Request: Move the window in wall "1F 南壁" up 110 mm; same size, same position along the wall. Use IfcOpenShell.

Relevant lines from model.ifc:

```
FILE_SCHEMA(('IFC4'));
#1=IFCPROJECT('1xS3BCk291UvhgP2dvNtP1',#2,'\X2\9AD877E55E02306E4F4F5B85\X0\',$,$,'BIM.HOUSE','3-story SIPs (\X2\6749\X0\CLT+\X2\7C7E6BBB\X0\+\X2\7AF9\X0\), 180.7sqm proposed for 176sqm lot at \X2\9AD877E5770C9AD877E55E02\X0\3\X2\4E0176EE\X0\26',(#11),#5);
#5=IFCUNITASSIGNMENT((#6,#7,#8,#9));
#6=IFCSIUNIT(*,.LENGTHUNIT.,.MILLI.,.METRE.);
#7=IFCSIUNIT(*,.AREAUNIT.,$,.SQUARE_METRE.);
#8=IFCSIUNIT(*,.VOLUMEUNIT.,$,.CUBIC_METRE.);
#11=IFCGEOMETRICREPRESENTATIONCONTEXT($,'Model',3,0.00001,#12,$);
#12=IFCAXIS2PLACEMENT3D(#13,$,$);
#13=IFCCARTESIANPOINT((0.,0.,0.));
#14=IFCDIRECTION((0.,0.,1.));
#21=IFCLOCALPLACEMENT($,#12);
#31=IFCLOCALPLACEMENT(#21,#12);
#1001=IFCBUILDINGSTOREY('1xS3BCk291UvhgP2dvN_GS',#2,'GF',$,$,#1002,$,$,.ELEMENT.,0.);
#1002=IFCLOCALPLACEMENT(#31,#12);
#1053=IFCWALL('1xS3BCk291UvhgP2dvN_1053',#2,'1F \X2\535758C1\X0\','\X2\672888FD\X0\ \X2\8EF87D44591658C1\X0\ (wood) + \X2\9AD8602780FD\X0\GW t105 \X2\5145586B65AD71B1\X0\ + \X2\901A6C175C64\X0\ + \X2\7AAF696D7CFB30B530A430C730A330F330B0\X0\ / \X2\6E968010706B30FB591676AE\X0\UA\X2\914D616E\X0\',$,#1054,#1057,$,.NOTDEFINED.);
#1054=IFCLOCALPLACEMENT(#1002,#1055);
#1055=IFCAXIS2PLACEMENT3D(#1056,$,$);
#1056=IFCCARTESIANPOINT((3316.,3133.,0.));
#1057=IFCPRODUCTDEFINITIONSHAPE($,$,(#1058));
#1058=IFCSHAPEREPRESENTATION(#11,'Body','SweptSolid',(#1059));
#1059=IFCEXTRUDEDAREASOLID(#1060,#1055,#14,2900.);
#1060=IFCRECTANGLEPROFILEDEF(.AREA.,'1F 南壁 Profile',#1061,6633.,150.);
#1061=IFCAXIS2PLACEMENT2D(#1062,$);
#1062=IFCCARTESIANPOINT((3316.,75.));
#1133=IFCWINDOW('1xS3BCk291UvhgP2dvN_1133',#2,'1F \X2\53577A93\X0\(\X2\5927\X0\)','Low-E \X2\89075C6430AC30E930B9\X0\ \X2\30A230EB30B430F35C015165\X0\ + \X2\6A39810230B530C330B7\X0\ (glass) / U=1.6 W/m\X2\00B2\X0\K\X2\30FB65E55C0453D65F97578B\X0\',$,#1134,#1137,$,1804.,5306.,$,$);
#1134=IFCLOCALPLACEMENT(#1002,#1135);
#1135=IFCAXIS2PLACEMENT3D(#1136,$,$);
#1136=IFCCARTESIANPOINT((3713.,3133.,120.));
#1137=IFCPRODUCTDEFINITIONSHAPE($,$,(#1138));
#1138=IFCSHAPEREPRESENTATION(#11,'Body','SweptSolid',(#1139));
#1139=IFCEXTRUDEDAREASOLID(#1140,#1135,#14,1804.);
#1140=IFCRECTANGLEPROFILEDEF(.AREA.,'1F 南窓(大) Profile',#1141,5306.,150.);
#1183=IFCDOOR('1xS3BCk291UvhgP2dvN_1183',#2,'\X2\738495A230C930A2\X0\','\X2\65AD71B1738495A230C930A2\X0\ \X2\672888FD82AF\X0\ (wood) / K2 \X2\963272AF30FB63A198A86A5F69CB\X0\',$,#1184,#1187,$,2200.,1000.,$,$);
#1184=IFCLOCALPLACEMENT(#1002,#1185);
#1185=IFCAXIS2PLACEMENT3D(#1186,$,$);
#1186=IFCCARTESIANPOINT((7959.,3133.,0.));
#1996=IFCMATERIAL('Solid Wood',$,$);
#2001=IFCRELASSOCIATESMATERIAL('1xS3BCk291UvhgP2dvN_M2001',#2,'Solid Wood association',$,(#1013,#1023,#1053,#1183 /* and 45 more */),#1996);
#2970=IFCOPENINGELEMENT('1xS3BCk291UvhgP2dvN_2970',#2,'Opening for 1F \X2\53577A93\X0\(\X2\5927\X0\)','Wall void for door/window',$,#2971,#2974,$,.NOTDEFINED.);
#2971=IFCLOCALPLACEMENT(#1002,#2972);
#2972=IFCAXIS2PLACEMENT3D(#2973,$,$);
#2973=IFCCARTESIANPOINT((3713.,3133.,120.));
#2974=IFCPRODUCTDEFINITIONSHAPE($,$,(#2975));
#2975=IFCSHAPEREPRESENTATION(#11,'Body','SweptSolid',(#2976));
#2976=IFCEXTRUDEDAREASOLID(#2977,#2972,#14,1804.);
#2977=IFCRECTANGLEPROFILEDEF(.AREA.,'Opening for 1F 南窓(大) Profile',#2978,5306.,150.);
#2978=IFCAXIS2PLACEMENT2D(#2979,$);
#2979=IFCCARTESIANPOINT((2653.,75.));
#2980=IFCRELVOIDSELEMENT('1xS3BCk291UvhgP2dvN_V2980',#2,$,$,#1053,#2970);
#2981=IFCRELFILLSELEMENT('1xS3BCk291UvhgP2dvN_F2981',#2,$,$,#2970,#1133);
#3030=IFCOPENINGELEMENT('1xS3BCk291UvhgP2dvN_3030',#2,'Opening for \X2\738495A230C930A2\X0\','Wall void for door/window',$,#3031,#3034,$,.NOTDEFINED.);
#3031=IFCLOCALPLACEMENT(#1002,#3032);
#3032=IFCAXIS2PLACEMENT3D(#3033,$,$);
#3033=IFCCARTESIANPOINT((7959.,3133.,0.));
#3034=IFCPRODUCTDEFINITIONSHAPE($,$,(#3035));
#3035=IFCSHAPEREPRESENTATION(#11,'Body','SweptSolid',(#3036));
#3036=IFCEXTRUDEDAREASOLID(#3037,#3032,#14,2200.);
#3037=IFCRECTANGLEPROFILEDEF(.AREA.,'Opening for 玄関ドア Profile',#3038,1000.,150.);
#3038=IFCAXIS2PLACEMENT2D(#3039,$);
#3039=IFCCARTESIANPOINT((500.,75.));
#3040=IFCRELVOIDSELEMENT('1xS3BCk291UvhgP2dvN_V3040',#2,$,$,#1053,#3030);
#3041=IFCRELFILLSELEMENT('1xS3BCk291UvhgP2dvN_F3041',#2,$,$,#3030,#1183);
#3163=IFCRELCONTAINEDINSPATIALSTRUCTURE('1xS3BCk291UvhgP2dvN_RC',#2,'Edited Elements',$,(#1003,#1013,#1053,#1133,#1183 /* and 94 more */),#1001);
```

```python
import numpy as np
import ifcopenshell
import ifcopenshell.api.geometry
import ifcopenshell.util.placement
import ifcopenshell.util.unit

model = ifcopenshell.open("model.ifc")
unit_scale = ifcopenshell.util.unit.calculate_unit_scale(model)

window = model.by_guid("1xS3BCk291UvhgP2dvN_1133")
opening = window.FillsVoids[0].RelatingOpeningElement
dz = 0.11 / unit_scale

shift = np.array([0.0, 0.0, dz])
# The window is not placed relative to its opening, so move both.
for product in (opening, window):
    matrix = ifcopenshell.util.placement.get_local_placement(product.ObjectPlacement)
    matrix[:3, 3] += shift
    ifcopenshell.api.geometry.edit_object_placement(model, product=product, matrix=matrix, is_si=False)

print(f"moved by {dz * unit_scale:+.3f} m")

model.write("model-out.ifc")
```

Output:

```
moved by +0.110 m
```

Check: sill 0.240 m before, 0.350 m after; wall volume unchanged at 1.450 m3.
